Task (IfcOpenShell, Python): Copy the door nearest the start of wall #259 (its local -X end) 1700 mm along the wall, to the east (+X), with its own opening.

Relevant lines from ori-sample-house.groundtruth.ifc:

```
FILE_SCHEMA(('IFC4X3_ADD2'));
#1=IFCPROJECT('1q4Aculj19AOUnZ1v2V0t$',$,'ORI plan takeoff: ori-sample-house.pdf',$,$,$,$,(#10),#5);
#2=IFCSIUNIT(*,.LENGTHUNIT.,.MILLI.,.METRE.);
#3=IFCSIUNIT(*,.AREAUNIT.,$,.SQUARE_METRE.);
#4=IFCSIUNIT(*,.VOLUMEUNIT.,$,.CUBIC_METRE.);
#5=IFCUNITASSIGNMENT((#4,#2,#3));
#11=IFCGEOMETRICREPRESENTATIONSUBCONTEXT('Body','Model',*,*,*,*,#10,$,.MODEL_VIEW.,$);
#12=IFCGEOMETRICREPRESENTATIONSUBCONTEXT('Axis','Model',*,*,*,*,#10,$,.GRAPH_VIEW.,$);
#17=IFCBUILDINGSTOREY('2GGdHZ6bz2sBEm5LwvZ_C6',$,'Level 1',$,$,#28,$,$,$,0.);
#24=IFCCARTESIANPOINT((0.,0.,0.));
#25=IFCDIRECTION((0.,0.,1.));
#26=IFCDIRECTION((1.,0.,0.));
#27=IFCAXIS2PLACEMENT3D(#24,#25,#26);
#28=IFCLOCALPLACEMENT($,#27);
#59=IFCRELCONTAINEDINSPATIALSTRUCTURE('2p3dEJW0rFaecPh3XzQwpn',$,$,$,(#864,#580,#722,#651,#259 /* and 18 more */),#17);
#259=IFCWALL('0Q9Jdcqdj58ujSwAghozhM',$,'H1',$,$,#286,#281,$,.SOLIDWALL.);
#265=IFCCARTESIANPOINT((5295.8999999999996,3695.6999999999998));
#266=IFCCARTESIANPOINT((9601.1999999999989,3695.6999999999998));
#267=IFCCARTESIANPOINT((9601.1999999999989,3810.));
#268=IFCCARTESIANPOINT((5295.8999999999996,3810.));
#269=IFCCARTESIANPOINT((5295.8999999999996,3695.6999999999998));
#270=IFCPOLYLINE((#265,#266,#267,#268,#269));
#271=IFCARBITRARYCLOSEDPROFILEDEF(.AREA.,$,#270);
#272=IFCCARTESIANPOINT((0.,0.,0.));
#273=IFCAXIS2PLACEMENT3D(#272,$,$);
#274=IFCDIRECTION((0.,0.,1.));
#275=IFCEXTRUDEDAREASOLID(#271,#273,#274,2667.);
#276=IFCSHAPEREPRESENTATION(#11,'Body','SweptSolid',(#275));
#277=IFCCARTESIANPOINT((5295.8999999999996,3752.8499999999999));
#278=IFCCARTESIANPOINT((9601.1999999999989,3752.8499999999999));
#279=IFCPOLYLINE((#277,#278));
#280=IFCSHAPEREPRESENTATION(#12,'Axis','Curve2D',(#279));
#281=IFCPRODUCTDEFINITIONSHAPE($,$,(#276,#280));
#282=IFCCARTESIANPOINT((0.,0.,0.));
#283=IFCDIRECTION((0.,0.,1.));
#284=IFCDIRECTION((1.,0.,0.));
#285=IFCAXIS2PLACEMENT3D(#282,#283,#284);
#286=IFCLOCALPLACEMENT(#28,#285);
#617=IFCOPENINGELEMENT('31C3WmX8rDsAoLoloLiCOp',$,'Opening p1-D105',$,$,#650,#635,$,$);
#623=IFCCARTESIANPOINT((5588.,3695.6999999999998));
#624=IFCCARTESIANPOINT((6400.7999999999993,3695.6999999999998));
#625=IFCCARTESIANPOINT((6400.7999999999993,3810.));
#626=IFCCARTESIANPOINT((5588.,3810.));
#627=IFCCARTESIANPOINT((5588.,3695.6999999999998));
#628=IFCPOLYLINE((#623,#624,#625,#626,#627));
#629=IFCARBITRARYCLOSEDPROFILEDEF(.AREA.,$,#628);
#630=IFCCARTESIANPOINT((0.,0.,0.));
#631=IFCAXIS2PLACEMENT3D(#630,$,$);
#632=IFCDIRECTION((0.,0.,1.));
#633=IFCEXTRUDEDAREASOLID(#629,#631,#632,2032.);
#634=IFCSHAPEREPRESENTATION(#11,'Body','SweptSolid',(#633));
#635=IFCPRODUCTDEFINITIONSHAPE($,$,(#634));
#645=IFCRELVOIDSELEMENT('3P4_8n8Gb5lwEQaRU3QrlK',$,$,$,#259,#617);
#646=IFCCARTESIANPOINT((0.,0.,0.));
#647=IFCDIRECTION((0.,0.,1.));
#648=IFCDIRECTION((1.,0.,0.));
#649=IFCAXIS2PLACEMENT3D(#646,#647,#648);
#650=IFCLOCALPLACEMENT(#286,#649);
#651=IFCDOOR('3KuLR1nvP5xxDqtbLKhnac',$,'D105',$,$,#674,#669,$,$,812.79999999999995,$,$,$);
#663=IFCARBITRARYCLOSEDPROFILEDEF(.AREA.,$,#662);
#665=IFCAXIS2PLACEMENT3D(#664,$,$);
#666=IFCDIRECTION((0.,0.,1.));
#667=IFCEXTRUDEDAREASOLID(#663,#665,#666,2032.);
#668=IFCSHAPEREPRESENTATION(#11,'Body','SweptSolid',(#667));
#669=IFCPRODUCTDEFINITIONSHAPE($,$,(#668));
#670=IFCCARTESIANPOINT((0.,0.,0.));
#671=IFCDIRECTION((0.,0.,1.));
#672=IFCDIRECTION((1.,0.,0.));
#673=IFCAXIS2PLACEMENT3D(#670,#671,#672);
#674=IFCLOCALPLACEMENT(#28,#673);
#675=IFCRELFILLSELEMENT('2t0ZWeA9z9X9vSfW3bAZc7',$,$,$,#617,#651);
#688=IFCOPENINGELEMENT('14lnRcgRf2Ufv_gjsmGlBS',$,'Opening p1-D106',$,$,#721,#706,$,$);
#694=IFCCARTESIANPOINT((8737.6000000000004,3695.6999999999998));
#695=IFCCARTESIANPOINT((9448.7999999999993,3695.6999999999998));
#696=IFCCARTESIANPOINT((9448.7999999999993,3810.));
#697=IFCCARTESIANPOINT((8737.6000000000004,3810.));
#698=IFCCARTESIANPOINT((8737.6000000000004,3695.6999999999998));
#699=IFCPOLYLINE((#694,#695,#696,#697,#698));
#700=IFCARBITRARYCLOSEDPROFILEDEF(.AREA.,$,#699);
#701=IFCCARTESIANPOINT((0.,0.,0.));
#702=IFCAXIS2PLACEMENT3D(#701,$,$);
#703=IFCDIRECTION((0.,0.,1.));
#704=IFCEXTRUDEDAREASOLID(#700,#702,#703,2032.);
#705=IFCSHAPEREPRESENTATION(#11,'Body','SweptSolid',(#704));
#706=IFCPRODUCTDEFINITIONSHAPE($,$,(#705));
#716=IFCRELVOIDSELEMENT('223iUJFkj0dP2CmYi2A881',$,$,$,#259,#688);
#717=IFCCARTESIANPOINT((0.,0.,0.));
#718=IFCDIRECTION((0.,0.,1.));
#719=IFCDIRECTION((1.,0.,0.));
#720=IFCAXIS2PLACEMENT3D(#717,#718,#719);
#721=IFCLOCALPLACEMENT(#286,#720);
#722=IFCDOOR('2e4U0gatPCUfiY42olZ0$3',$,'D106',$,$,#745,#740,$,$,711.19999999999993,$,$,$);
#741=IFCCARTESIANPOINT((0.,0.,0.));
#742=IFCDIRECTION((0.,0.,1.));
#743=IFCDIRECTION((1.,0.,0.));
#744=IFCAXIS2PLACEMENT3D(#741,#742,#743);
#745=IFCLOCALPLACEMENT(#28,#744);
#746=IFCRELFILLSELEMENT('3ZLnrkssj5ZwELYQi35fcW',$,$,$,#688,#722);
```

```python
import ifcopenshell
import ifcopenshell.api.feature
import ifcopenshell.api.geometry
import ifcopenshell.api.root
import ifcopenshell.geom
import ifcopenshell.util.element
import ifcopenshell.util.placement
import ifcopenshell.util.shape
import ifcopenshell.util.unit

model = ifcopenshell.open("ori-sample-house.groundtruth.ifc")
unit_scale = ifcopenshell.util.unit.calculate_unit_scale(model)
settings = ifcopenshell.geom.settings()


def volume(element):
    """Net volume in cubic metres, openings subtracted."""
    shape = ifcopenshell.geom.create_shape(settings, element)
    return ifcopenshell.util.shape.get_volume(shape.geometry)


door = model.by_id(651)
opening = door.FillsVoids[0].RelatingOpeningElement
wall = opening.VoidsElements[0].RelatingBuildingElement
before = volume(wall)
shift = ifcopenshell.util.placement.get_local_placement(wall.ObjectPlacement)[:3, 0] * 1.7 / unit_scale

# copy_class copies the void relationship, type, container and properties, but no geometry.
new_opening = ifcopenshell.api.root.copy_class(model, product=opening)
new_opening.Representation = ifcopenshell.util.element.copy_deep(
    model, opening.Representation, exclude=["IfcGeometricRepresentationContext", "IfcRepresentationMap"]
)
new_door = ifcopenshell.api.root.copy_class(model, product=door)
new_door.Representation = ifcopenshell.util.element.copy_deep(
    model, door.Representation, exclude=["IfcGeometricRepresentationContext", "IfcRepresentationMap"]
)
ifcopenshell.api.feature.add_filling(model, opening=new_opening, element=new_door)

for old, new in ((opening, new_opening), (door, new_door)):
    matrix = ifcopenshell.util.placement.get_local_placement(old.ObjectPlacement)
    matrix[:3, 3] += shift
    ifcopenshell.api.geometry.edit_object_placement(model, product=new, matrix=matrix, is_si=False)

after = volume(wall)

print(f"wall volume {before:.3f} -> {after:.3f} m3")

model.write("ori-sample-house.groundtruth_v2.ifc")
```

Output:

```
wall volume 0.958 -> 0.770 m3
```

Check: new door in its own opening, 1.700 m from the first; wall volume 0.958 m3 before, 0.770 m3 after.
